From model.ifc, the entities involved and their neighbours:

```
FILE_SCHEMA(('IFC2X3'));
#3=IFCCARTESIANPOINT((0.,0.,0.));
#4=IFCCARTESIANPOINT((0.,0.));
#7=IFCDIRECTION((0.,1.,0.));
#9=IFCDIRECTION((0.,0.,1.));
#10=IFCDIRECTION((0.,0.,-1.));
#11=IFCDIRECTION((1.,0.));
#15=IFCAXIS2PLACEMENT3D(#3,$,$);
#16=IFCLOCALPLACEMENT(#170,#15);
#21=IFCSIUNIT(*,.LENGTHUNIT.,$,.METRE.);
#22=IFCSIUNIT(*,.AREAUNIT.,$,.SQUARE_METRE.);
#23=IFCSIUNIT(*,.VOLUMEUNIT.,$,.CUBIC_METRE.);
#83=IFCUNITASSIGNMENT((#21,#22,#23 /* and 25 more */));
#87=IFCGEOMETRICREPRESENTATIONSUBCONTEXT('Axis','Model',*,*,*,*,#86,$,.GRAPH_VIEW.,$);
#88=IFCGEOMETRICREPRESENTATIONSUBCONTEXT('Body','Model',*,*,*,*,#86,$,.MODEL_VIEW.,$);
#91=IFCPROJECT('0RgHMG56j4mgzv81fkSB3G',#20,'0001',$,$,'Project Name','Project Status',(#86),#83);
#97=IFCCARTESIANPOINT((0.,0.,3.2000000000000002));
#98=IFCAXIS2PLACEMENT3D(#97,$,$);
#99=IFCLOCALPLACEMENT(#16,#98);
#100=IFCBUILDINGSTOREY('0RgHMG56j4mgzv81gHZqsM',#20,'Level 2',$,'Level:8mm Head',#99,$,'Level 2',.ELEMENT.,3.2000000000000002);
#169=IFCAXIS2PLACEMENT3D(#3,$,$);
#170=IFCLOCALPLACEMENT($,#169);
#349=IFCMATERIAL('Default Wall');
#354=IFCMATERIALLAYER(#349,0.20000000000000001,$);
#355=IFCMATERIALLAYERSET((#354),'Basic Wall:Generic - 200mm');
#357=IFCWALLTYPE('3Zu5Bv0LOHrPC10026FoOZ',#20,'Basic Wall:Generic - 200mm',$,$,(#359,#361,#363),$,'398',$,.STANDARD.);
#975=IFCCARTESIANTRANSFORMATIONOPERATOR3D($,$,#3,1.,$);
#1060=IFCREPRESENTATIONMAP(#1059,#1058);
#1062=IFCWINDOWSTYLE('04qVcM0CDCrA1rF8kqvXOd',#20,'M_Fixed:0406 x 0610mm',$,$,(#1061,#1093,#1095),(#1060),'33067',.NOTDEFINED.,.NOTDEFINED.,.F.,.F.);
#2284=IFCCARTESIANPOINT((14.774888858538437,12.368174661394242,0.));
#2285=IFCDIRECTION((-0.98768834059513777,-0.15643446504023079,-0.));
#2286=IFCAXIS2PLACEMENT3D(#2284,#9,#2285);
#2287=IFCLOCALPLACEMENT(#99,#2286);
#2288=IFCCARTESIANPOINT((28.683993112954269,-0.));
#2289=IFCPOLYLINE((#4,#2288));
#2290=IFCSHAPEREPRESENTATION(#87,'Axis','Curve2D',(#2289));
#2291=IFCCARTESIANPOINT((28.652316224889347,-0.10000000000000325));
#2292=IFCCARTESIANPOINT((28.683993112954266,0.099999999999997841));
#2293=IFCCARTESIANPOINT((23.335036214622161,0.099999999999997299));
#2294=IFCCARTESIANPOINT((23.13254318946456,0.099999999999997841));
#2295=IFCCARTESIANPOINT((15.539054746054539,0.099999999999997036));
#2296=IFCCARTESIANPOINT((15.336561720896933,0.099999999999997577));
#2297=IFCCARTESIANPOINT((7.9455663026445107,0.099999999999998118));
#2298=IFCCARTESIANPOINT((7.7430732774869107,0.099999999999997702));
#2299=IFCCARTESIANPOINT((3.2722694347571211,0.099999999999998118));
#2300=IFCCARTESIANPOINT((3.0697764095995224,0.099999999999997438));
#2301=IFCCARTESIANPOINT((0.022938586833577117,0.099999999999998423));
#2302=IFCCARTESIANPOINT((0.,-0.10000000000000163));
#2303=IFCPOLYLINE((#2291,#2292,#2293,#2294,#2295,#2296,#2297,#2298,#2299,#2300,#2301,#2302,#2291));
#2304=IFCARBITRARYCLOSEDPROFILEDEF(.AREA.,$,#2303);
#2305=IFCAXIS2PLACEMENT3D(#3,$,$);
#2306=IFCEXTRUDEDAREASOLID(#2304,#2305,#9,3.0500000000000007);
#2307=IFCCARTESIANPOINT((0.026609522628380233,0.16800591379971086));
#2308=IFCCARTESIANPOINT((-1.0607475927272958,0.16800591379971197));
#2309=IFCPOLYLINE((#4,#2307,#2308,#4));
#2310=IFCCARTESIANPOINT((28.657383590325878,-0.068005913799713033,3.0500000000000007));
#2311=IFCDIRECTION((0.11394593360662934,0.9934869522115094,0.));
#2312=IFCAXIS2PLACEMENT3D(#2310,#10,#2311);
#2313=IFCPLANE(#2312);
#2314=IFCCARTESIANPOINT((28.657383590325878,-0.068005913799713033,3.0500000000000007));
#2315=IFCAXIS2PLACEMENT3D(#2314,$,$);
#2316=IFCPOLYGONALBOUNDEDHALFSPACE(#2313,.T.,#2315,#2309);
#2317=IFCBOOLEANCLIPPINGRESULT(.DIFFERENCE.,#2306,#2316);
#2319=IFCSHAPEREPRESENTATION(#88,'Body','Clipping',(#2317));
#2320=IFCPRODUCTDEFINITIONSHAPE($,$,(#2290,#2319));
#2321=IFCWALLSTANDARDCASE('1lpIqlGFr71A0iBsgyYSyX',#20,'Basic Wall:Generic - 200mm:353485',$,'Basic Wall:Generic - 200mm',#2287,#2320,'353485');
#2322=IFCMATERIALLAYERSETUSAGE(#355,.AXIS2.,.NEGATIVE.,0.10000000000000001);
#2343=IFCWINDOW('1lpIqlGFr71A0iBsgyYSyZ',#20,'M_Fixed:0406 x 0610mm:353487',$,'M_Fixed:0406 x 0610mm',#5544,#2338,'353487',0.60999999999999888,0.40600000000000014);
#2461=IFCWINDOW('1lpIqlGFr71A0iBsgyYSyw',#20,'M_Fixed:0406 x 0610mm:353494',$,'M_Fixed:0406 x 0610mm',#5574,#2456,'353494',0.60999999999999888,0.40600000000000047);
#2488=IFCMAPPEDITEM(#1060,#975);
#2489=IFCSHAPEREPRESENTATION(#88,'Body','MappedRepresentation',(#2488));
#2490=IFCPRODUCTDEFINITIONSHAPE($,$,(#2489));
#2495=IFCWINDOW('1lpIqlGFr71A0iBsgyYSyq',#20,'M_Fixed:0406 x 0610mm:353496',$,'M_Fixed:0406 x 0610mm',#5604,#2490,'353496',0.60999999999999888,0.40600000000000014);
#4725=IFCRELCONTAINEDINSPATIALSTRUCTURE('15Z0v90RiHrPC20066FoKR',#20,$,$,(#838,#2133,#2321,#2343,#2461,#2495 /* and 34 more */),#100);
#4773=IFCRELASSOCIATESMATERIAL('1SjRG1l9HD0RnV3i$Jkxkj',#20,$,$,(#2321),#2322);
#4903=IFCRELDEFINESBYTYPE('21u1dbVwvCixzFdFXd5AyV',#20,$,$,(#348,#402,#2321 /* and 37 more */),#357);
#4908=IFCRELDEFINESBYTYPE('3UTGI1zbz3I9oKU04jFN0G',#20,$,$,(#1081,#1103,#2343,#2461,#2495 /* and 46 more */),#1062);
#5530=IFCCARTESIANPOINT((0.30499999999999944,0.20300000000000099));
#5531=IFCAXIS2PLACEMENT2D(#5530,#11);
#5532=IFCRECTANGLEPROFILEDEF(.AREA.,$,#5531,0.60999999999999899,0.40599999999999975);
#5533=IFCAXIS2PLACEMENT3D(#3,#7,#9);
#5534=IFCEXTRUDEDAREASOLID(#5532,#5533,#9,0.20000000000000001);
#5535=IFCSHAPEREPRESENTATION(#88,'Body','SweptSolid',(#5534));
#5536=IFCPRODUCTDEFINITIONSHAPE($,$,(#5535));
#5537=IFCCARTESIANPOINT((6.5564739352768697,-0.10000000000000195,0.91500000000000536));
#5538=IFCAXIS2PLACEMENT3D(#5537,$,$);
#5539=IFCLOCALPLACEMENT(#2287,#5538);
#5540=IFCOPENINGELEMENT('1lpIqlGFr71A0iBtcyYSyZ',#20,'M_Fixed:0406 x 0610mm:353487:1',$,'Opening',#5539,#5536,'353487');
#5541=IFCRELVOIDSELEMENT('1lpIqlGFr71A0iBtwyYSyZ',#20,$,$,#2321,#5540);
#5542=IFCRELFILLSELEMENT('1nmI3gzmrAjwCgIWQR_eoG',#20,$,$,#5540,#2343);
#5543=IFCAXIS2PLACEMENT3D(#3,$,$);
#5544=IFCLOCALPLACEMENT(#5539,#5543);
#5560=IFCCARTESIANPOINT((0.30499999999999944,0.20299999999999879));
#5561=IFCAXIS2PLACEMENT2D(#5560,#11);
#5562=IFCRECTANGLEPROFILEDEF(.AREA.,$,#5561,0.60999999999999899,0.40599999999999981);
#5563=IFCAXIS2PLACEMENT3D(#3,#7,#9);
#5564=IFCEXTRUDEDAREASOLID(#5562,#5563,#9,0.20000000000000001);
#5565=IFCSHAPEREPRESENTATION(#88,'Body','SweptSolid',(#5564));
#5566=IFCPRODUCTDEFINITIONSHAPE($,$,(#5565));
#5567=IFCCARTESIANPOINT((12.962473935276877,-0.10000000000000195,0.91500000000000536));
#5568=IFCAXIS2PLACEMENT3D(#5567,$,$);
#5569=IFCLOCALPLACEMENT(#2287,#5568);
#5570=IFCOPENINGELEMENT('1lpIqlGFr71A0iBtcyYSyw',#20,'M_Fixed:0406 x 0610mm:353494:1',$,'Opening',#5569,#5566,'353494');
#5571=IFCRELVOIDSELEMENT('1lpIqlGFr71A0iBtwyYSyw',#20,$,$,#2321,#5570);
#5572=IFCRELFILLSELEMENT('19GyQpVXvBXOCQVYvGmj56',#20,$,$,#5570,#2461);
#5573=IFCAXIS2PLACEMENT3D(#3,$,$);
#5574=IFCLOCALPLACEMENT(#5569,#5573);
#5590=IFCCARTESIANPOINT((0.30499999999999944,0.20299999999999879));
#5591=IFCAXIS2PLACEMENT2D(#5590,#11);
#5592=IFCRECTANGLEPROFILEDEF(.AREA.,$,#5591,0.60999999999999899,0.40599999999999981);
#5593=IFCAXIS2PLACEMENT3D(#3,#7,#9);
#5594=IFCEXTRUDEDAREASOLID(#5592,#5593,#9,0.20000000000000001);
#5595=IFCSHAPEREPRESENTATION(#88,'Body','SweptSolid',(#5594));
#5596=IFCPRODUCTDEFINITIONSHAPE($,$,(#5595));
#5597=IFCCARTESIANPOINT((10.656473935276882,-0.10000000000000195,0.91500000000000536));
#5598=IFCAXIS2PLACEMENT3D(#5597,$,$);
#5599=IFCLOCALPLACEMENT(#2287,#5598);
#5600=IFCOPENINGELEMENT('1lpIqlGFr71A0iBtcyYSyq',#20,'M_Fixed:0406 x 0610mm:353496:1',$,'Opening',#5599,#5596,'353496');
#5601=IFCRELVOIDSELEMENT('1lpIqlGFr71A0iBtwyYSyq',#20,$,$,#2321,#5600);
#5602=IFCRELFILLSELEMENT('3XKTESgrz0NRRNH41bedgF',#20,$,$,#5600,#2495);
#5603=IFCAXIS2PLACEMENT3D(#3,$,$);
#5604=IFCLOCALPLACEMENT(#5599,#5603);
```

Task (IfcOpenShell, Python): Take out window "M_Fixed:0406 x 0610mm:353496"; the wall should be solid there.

```python
import ifcopenshell
import ifcopenshell.api.feature
import ifcopenshell.api.root
import ifcopenshell.geom
import ifcopenshell.util.shape

model = ifcopenshell.open("model.ifc")
settings = ifcopenshell.geom.settings()


def volume(element):
    """Net volume in cubic metres, openings subtracted."""
    shape = ifcopenshell.geom.create_shape(settings, element)
    return ifcopenshell.util.shape.get_volume(shape.geometry)


window = model.by_guid("1lpIqlGFr71A0iBsgyYSyq")
opening = window.FillsVoids[0].RelatingOpeningElement
wall = opening.VoidsElements[0].RelatingBuildingElement
before = volume(wall)

ifcopenshell.api.root.remove_product(model, product=window)
ifcopenshell.api.feature.remove_feature(model, feature=opening)

after = volume(wall)

print(f"wall volume {before:.3f} -> {after:.3f} m3")

model.write("model_edited.ifc")
```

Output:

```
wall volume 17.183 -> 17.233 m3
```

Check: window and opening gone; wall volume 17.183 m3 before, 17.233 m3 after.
